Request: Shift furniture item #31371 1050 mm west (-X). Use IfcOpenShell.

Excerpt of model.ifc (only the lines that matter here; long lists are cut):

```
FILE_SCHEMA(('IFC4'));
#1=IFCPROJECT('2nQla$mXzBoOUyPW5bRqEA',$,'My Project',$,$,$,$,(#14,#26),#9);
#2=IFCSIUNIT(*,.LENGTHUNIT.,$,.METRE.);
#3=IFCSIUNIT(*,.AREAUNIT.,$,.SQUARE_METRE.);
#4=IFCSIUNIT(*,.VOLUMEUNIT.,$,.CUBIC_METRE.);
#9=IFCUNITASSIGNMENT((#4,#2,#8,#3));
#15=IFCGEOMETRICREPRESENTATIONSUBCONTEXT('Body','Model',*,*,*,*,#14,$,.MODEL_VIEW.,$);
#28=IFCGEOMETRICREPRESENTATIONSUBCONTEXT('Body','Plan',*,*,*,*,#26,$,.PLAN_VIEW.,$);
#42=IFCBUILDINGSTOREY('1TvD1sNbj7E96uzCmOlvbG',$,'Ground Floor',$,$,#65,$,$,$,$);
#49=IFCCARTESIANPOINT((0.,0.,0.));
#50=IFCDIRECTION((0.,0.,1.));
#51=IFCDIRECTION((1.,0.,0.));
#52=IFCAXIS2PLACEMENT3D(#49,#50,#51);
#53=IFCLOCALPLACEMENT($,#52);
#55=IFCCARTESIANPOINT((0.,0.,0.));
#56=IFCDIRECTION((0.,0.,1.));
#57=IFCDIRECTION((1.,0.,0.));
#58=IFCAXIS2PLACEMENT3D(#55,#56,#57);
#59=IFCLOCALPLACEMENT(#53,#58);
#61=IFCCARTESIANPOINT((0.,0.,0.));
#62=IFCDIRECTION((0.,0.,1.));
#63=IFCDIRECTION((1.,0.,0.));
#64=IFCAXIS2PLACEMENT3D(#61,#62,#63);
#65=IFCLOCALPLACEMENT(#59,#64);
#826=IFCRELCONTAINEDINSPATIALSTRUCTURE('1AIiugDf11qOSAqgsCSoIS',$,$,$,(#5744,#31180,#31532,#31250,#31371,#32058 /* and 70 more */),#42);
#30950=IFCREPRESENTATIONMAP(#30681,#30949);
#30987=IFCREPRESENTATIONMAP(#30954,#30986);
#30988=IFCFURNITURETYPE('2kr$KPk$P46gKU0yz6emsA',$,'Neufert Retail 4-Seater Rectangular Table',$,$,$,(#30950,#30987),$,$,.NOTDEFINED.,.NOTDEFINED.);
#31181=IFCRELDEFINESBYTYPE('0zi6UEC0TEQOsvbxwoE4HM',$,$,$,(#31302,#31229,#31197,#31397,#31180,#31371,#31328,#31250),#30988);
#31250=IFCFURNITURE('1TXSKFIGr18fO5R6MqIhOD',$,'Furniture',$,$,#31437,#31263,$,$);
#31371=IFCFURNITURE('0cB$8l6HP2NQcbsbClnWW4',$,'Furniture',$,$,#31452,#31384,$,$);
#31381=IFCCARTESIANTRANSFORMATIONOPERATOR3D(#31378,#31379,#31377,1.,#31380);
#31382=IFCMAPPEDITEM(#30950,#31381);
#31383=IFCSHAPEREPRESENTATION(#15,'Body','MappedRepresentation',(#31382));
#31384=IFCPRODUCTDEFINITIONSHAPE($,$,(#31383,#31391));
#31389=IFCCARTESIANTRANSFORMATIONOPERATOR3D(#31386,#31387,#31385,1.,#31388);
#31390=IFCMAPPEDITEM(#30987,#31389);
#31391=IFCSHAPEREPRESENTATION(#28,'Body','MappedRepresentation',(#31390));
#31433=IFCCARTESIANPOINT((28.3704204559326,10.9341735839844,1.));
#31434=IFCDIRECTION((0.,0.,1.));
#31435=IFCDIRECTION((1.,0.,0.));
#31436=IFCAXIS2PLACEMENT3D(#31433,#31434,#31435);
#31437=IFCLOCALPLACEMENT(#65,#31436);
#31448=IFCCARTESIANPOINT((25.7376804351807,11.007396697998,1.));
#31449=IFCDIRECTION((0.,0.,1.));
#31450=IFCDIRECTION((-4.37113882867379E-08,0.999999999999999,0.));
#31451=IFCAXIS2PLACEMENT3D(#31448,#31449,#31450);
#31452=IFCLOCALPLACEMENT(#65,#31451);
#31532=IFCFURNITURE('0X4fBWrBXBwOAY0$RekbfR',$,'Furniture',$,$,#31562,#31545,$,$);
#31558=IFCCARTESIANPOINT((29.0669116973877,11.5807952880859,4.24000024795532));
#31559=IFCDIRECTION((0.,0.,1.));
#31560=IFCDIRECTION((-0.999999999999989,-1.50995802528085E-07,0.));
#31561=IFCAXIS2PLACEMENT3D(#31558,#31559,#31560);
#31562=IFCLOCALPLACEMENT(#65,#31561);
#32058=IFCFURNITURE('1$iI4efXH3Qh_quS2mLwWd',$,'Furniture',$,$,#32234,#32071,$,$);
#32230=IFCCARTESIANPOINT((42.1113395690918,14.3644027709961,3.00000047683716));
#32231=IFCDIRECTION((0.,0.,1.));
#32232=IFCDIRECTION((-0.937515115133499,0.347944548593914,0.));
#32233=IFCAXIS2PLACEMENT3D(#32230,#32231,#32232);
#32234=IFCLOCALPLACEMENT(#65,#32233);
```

```python
import ifcopenshell
import ifcopenshell.api.geometry
import ifcopenshell.util.placement

model = ifcopenshell.open("model.ifc")

item = model.by_guid("0cB$8l6HP2NQcbsbClnWW4")
matrix = ifcopenshell.util.placement.get_local_placement(item.ObjectPlacement)
matrix[0, 3] -= 1.05
ifcopenshell.api.geometry.edit_object_placement(model, product=item, matrix=matrix, is_si=False)

print(ifcopenshell.util.placement.get_local_placement(item.ObjectPlacement).round(3) + 0.0)

model.write("model_updated.ifc")
```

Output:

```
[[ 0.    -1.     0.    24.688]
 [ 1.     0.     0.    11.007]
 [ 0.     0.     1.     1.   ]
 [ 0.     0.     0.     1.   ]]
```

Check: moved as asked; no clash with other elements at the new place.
